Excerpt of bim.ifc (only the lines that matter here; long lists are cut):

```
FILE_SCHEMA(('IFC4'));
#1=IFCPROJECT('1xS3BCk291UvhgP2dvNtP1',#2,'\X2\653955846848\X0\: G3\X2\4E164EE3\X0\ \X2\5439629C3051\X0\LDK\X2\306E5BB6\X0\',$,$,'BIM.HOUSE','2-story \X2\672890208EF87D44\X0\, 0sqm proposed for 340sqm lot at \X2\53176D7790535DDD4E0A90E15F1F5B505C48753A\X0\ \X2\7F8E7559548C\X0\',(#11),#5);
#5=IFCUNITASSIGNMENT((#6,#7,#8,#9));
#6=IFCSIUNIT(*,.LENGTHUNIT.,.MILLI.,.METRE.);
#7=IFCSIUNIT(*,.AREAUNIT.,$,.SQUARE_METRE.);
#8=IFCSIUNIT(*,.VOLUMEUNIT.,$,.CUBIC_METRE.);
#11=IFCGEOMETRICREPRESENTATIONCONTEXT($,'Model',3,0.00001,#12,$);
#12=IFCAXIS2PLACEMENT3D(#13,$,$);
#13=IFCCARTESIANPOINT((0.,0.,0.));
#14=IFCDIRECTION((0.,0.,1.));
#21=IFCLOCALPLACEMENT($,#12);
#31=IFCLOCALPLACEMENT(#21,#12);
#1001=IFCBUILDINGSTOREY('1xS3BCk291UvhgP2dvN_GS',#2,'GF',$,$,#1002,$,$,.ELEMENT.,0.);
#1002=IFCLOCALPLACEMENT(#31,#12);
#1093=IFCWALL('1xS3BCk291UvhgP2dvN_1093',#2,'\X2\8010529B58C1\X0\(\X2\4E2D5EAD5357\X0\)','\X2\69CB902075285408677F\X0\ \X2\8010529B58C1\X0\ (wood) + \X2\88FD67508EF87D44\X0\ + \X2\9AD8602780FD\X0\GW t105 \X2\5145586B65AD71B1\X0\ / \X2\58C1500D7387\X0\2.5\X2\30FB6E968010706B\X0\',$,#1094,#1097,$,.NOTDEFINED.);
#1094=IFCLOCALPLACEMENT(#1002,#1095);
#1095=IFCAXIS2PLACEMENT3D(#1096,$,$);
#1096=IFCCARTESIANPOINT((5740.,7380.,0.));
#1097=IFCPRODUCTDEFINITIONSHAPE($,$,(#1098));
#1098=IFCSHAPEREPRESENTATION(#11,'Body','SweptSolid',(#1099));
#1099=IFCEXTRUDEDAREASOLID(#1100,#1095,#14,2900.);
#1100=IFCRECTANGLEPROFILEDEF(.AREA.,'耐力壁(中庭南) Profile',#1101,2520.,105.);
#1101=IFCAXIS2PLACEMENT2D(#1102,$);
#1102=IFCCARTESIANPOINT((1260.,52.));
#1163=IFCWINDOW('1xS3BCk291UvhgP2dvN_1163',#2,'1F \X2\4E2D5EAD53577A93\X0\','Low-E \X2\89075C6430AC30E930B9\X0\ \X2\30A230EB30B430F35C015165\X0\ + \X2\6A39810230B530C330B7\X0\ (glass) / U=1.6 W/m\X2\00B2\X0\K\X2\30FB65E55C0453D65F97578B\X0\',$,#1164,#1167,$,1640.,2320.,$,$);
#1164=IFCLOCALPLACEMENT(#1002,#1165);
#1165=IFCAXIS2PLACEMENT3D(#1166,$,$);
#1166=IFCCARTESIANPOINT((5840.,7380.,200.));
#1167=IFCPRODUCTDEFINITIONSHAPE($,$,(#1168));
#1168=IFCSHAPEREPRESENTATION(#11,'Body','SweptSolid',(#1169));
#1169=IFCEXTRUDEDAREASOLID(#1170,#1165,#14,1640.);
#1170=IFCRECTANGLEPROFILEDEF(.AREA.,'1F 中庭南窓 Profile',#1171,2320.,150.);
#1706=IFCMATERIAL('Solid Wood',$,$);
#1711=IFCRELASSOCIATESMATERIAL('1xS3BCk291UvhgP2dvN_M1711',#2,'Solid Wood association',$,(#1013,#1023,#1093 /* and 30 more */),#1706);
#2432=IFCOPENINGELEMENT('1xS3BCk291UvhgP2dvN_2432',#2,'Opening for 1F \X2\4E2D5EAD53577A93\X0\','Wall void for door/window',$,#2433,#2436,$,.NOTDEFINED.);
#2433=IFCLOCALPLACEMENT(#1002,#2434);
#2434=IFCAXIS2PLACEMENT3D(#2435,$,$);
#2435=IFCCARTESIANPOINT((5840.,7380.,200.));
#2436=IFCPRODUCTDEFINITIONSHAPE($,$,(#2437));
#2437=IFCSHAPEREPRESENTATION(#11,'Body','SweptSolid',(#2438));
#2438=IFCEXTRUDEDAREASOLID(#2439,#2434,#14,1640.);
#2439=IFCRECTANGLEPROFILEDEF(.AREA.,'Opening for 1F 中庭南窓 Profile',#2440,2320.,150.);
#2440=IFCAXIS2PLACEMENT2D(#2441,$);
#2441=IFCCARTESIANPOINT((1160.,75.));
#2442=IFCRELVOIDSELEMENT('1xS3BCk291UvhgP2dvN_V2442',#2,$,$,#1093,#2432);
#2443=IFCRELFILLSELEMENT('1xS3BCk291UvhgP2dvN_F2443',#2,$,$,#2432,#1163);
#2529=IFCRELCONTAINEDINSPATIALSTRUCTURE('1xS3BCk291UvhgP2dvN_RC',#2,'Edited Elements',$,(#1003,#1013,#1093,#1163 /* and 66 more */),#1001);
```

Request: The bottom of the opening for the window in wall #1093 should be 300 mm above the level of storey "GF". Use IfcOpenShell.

```python
import numpy as np
import ifcopenshell
import ifcopenshell.api.geometry
import ifcopenshell.geom
import ifcopenshell.util.element
import ifcopenshell.util.placement
import ifcopenshell.util.shape
import ifcopenshell.util.unit

model = ifcopenshell.open("bim.ifc")
unit_scale = ifcopenshell.util.unit.calculate_unit_scale(model)

window = model.by_id(1163)
opening = window.FillsVoids[0].RelatingOpeningElement
storey = ifcopenshell.util.element.get_container(window, ifc_class="IfcBuildingStorey")
level = ifcopenshell.util.placement.get_local_placement(storey.ObjectPlacement)[2, 3]

# The opening's origin need not be at the sill, so measure its lowest point.
shape = ifcopenshell.geom.create_shape(ifcopenshell.geom.settings(), opening)
bottom = ifcopenshell.util.shape.get_shape_bottom_elevation(shape, shape.geometry) / unit_scale
dz = level + 0.3 / unit_scale - bottom

shift = np.array([0.0, 0.0, dz])
# The window is not placed relative to its opening, so move both.
for product in (opening, window):
    matrix = ifcopenshell.util.placement.get_local_placement(product.ObjectPlacement)
    matrix[:3, 3] += shift
    ifcopenshell.api.geometry.edit_object_placement(model, product=product, matrix=matrix, is_si=False)

print(f"moved by {dz * unit_scale:+.3f} m")

model.write("bim-out.ifc")
```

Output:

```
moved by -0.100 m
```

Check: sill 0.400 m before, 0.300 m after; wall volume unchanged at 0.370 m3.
